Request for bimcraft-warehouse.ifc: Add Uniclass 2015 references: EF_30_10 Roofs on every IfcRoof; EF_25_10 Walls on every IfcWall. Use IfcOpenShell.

First a look at what the model holds.

```python
import ifcopenshell

model = ifcopenshell.open("bimcraft-warehouse.ifc")
print(model.schema)
print("classifications:", [c.Name for c in model.by_type("IfcClassification")])
for ifc_class in ("IfcDoor", "IfcRoof", "IfcStair", "IfcWall", "IfcWindow"):
    print(ifc_class, len(model.by_type(ifc_class)))
```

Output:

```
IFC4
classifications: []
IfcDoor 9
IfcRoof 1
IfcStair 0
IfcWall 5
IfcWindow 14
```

```python
import ifcopenshell
import ifcopenshell.api.classification

model = ifcopenshell.open("bimcraft-warehouse.ifc")

system = ifcopenshell.api.classification.add_classification(model, classification="Uniclass 2015")

codes = {
    "IfcRoof": ("EF_30_10", "Roofs"),
    "IfcWall": ("EF_25_10", "Walls"),
}
for ifc_class, (code, name) in codes.items():
    products = model.by_type(ifc_class)
    ifcopenshell.api.classification.add_reference(
        model, products=products, classification=system, identification=code, name=name
    )
    print(code, len(products))

model.write("bimcraft-warehouse_rev.ifc")
```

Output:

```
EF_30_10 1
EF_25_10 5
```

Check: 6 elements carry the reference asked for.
